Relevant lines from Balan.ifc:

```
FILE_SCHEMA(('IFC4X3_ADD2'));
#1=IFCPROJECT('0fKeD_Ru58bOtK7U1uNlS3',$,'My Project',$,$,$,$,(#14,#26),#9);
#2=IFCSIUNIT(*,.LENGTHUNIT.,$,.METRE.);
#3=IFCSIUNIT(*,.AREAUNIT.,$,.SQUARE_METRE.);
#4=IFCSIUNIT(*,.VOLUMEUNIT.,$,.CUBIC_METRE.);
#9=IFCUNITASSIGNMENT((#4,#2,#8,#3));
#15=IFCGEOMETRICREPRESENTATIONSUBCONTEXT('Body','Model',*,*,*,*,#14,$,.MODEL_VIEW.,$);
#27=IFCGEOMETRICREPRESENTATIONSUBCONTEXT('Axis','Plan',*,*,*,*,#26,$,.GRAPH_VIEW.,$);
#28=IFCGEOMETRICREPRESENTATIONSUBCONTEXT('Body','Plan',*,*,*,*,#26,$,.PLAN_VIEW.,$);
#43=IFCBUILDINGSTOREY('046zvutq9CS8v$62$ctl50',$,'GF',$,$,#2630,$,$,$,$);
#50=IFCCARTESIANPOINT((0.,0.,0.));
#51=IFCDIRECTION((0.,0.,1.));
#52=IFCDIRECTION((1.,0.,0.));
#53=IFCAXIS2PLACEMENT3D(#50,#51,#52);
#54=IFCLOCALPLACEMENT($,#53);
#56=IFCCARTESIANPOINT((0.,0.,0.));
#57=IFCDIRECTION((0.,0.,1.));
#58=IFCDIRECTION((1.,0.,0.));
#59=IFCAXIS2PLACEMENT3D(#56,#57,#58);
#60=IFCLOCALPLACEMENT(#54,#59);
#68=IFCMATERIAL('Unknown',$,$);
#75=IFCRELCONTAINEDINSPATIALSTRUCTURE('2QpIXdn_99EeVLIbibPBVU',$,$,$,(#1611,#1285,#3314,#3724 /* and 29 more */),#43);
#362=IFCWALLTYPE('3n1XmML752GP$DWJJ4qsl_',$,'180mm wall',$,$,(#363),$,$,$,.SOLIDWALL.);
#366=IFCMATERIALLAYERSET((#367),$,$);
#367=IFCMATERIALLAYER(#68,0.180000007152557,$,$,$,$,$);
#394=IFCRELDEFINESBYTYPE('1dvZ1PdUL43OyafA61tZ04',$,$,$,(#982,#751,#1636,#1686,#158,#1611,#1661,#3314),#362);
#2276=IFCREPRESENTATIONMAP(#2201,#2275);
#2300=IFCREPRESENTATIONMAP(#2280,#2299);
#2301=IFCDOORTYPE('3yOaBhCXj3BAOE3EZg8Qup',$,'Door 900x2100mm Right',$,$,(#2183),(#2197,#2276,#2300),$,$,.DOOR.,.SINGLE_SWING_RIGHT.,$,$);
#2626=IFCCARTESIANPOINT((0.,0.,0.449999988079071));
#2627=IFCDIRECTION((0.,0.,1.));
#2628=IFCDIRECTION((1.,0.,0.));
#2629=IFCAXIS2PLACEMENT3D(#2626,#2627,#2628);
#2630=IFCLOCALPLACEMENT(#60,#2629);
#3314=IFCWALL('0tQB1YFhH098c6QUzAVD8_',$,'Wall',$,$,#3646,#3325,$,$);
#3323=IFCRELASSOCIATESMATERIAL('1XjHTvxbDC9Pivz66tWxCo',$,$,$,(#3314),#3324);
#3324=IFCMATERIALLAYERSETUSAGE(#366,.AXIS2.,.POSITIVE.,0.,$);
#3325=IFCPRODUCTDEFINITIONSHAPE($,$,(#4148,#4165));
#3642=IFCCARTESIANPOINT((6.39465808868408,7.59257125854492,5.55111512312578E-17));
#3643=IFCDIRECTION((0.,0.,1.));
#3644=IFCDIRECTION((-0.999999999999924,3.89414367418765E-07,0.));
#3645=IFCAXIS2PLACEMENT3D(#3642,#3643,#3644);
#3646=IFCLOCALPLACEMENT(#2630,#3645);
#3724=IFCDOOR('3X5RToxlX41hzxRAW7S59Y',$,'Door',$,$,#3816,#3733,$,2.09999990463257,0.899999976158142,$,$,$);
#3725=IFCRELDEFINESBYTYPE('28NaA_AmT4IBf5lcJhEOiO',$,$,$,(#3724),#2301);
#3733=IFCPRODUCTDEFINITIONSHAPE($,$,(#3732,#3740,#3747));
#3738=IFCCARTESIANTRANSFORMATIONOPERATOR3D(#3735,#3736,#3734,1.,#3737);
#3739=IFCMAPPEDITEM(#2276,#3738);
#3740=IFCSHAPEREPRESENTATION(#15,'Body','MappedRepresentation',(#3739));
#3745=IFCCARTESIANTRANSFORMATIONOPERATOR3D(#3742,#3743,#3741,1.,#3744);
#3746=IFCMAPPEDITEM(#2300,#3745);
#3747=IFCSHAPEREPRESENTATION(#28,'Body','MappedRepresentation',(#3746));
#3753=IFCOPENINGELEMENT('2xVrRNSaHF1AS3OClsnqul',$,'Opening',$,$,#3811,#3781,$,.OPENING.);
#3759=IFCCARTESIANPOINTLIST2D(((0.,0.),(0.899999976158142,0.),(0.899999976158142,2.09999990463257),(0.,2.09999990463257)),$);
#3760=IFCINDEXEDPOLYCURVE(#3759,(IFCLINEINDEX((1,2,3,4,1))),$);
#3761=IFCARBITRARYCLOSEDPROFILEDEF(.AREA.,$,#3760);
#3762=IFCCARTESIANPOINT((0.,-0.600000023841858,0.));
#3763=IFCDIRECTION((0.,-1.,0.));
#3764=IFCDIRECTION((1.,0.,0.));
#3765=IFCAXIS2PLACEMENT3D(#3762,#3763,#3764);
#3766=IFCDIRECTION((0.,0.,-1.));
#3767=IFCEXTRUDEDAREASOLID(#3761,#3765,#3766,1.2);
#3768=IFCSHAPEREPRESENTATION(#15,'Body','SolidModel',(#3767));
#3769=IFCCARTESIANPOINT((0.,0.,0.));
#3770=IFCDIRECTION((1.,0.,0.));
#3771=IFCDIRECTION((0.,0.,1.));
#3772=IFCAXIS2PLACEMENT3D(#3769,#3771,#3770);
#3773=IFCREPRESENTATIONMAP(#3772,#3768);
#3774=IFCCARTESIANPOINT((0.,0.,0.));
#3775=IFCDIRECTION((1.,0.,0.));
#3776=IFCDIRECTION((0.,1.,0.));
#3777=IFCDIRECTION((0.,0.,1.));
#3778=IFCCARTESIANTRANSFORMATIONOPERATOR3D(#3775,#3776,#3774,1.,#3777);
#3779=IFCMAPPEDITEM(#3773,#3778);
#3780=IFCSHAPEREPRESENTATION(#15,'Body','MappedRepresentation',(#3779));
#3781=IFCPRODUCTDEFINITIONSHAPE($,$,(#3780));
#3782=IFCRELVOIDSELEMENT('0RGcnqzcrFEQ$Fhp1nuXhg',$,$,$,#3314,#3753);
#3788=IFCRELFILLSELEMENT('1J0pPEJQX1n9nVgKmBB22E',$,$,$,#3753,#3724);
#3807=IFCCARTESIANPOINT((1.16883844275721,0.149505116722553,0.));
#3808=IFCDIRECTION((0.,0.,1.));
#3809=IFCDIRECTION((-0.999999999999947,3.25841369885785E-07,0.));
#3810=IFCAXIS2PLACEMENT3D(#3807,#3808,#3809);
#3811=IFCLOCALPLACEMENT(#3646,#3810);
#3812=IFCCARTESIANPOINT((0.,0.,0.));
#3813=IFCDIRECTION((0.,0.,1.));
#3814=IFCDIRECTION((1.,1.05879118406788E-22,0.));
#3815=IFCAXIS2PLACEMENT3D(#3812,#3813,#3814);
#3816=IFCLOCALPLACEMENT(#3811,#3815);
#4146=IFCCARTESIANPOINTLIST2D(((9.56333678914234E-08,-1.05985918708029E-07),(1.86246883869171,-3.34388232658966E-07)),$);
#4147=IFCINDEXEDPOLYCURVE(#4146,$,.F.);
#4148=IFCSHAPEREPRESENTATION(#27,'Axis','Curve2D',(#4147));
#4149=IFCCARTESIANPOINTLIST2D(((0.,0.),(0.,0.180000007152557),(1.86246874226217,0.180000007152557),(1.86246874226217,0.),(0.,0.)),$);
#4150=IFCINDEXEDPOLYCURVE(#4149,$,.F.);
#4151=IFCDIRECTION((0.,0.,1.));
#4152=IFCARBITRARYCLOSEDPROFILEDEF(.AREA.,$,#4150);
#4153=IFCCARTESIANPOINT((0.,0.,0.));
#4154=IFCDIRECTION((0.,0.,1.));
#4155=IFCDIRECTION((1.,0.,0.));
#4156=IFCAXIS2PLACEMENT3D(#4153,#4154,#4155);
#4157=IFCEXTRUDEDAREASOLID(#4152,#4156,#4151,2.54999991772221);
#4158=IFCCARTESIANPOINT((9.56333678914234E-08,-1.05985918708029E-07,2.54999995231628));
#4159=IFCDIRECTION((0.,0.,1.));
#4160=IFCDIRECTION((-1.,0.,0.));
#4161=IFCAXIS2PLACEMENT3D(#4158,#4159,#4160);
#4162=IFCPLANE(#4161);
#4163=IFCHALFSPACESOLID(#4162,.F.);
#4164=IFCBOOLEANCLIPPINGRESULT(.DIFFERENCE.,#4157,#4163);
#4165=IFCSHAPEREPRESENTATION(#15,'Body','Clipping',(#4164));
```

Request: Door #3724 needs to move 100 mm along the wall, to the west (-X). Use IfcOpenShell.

```python
import ifcopenshell
import ifcopenshell.api.geometry
import ifcopenshell.util.placement

model = ifcopenshell.open("Balan.ifc")

door = model.by_guid("3X5RToxlX41hzxRAW7S59Y")
opening = door.FillsVoids[0].RelatingOpeningElement
wall = opening.VoidsElements[0].RelatingBuildingElement

wall_matrix = ifcopenshell.util.placement.get_local_placement(wall.ObjectPlacement)
shift = wall_matrix[:3, 0] * 0.1
before = ifcopenshell.util.placement.get_local_placement(door.ObjectPlacement)[:3, 3].copy()

# The door is placed relative to its opening, so it follows when the opening moves.
matrix = ifcopenshell.util.placement.get_local_placement(opening.ObjectPlacement)
matrix[:3, 3] += shift
ifcopenshell.api.geometry.edit_object_placement(
    model, product=opening, matrix=matrix, is_si=False, should_transform_children=True
)

after = ifcopenshell.util.placement.get_local_placement(door.ObjectPlacement)[:3, 3]
print("door moved by", (after - before).round(3) + 0.0)

model.write("Balan_rev.ifc")
```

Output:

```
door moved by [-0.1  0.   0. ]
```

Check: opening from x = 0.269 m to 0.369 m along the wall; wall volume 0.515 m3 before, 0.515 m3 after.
